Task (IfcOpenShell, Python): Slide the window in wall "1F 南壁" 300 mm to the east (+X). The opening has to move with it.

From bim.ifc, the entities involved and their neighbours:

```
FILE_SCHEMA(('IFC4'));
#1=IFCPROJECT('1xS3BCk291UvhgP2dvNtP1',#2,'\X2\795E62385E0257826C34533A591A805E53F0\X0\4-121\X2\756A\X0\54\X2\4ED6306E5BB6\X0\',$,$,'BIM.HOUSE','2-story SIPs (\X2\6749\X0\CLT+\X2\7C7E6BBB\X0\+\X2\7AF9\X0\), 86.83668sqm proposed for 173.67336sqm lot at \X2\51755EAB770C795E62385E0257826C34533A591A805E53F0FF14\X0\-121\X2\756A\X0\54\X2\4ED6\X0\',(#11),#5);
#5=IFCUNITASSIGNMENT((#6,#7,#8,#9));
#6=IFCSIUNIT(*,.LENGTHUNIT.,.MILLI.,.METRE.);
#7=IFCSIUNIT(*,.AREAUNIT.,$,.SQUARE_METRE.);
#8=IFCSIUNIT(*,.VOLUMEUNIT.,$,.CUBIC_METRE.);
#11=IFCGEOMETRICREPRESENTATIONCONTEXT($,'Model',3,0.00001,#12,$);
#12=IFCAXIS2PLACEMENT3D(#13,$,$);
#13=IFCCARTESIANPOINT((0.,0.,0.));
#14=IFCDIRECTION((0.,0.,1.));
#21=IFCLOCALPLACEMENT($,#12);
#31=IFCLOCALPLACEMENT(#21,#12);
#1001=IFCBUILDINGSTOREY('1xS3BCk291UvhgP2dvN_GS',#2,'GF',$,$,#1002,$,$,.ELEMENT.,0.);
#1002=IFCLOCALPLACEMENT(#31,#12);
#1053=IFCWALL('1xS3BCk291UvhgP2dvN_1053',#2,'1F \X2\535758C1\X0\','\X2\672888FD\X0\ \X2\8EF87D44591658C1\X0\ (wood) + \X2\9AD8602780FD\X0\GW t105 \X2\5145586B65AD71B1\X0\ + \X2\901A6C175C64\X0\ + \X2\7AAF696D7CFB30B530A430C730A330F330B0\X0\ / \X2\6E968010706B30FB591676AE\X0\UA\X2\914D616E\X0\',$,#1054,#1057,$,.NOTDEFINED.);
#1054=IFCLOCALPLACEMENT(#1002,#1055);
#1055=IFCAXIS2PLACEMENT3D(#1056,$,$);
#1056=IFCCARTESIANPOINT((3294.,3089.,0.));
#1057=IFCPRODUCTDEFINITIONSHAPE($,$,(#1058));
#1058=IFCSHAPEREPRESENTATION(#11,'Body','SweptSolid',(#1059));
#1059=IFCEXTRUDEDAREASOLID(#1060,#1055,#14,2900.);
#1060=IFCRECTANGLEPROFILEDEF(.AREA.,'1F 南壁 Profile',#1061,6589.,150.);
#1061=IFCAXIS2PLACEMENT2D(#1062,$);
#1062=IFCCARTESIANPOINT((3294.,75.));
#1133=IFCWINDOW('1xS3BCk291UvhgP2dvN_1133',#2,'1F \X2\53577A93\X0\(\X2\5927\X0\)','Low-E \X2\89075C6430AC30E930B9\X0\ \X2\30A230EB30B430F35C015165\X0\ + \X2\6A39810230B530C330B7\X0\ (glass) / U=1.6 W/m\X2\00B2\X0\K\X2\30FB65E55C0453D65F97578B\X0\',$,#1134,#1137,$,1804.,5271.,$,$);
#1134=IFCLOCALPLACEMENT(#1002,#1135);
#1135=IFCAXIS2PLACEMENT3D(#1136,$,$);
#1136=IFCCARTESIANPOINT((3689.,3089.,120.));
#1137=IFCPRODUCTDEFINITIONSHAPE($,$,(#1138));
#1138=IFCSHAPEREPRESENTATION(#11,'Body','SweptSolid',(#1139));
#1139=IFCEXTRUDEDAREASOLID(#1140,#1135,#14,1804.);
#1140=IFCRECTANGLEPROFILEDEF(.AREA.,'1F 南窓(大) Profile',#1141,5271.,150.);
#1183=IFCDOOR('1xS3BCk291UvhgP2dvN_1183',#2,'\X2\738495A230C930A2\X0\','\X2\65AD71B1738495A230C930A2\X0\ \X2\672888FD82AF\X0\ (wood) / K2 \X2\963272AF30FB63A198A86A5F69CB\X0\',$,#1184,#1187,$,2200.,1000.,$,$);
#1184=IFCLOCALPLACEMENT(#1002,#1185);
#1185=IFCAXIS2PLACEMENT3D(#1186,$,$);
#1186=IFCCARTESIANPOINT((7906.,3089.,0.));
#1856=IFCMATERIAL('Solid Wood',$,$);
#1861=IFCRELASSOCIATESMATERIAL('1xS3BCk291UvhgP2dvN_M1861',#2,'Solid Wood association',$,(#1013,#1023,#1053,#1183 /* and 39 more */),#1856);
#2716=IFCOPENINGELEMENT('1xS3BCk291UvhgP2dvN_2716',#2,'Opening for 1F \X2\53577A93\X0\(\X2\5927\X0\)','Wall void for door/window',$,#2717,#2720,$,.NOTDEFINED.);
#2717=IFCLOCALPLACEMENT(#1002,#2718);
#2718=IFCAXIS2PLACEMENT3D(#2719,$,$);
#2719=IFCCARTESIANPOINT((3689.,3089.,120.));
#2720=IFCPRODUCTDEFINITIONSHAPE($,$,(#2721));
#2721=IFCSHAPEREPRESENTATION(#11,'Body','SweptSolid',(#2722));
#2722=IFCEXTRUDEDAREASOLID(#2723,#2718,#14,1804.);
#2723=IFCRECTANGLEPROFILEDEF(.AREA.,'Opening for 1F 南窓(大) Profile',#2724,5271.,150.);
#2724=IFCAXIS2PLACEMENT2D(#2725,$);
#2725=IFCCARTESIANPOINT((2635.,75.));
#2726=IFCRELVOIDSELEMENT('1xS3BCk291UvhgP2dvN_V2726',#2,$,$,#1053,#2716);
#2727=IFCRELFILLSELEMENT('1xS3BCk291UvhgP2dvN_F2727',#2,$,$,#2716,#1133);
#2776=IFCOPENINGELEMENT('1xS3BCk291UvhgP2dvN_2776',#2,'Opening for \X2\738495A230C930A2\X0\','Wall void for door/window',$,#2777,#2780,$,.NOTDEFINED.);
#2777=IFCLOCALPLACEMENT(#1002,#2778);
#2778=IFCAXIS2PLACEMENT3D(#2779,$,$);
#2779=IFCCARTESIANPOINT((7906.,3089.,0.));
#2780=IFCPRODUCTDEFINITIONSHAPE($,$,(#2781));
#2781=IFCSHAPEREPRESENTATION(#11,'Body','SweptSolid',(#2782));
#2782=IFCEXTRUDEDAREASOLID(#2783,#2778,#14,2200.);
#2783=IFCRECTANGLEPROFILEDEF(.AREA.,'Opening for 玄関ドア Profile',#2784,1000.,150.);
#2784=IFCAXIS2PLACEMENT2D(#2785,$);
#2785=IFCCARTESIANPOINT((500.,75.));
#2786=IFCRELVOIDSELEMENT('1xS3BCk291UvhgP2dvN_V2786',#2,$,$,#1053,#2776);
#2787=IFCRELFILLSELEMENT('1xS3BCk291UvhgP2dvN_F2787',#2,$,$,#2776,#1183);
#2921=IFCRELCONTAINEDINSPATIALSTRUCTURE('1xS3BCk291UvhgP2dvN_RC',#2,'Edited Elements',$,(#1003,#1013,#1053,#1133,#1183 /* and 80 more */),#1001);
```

```python
import ifcopenshell
import ifcopenshell.api.geometry
import ifcopenshell.util.placement
import ifcopenshell.util.unit

model = ifcopenshell.open("bim.ifc")
unit_scale = ifcopenshell.util.unit.calculate_unit_scale(model)

window = model.by_id(1133)
opening = window.FillsVoids[0].RelatingOpeningElement
wall = opening.VoidsElements[0].RelatingBuildingElement

wall_matrix = ifcopenshell.util.placement.get_local_placement(wall.ObjectPlacement)
shift = wall_matrix[:3, 0] * 0.3 / unit_scale
before = ifcopenshell.util.placement.get_local_placement(window.ObjectPlacement)[:3, 3].copy()

# The window is not placed relative to its opening, so move both.
for product in (opening, window):
    matrix = ifcopenshell.util.placement.get_local_placement(product.ObjectPlacement)
    matrix[:3, 3] += shift
    ifcopenshell.api.geometry.edit_object_placement(model, product=product, matrix=matrix, is_si=False)

after = ifcopenshell.util.placement.get_local_placement(window.ObjectPlacement)[:3, 3]
print("window moved by", (after - before).round(3) + 0.0)

model.write("bim_rev.ifc")
```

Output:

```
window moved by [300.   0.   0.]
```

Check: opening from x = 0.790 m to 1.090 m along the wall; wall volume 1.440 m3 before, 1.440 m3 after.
